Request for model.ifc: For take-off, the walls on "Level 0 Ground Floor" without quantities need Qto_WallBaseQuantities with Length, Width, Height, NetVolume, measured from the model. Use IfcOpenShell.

First a look at what the model holds.

```python
import ifcopenshell
import ifcopenshell.util.element
import ifcopenshell.util.unit

model = ifcopenshell.open("model.ifc")
print(model.schema)
for unit_type in ("LENGTHUNIT", "AREAUNIT", "VOLUMEUNIT"):
    print(unit_type, ifcopenshell.util.unit.calculate_unit_scale(model, unit_type))
storey = next(s for s in model.by_type("IfcBuildingStorey") if s.Name == "Level 0 Ground Floor")
walls = [e for e in ifcopenshell.util.element.get_decomposition(storey) if e.is_a("IfcWall")]
for e in sorted(walls, key=lambda e: e.id()):
    print(e.id(), e.is_a(), e.Name, list(ifcopenshell.util.element.get_psets(e, qtos_only=True)), sep=" | ")
```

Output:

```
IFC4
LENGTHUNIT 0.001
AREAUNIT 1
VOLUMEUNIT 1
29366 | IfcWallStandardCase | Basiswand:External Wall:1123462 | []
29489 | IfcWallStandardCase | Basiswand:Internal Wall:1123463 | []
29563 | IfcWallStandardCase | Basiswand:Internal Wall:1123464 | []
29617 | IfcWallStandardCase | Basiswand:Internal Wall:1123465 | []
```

```python
import ifcopenshell
import ifcopenshell.api.pset
import ifcopenshell.geom
import ifcopenshell.util.element
import ifcopenshell.util.shape
import ifcopenshell.util.unit

model = ifcopenshell.open("model.ifc")
unit_scale = ifcopenshell.util.unit.calculate_unit_scale(model)
volume_scale = ifcopenshell.util.unit.calculate_unit_scale(model, "VOLUMEUNIT")
settings = ifcopenshell.geom.settings()

storey = next(s for s in model.by_type("IfcBuildingStorey") if s.Name == "Level 0 Ground Floor")
walls = [e for e in ifcopenshell.util.element.get_decomposition(storey) if e.is_a("IfcWall")]

for e in sorted(walls, key=lambda e: e.id()):
    if ifcopenshell.util.element.get_psets(e, qtos_only=True, should_inherit=False):
        continue
    # Geometry comes back in metres, in the element's own axes.
    shape = ifcopenshell.geom.create_shape(settings, e)
    values = {
        "Length": ifcopenshell.util.shape.get_x(shape.geometry) / unit_scale,
        "Width": ifcopenshell.util.shape.get_y(shape.geometry) / unit_scale,
        "Height": ifcopenshell.util.shape.get_z(shape.geometry) / unit_scale,
        "NetVolume": ifcopenshell.util.shape.get_volume(shape.geometry) / volume_scale,
    }
    qto = ifcopenshell.api.pset.add_qto(model, product=e, name="Qto_WallBaseQuantities")
    ifcopenshell.api.pset.edit_qto(model, qto=qto, properties=values)
    print(e.id(), {k: round(v, 3) for k, v in values.items()})

model.write("model-out.ifc")
```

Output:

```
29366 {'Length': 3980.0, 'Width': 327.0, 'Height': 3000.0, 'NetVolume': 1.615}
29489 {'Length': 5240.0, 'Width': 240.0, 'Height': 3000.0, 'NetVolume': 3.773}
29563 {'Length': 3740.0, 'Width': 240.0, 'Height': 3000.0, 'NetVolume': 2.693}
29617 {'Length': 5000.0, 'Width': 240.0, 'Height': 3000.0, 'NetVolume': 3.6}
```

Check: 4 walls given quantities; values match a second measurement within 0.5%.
